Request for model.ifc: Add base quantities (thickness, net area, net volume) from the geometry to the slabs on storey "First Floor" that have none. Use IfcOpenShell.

First a look at what the model holds.

```python
import ifcopenshell
import ifcopenshell.util.element
import ifcopenshell.util.unit

model = ifcopenshell.open("model.ifc")
print(model.schema)
for unit_type in ("LENGTHUNIT", "AREAUNIT", "VOLUMEUNIT"):
    print(unit_type, ifcopenshell.util.unit.calculate_unit_scale(model, unit_type))
storey = next(s for s in model.by_type("IfcBuildingStorey") if s.Name == "First Floor")
slabs = [e for e in ifcopenshell.util.element.get_decomposition(storey) if e.is_a("IfcSlab")]
for e in sorted(slabs, key=lambda e: e.id()):
    print(e.id(), e.is_a(), e.Name, list(ifcopenshell.util.element.get_psets(e, qtos_only=True)), sep=" | ")
```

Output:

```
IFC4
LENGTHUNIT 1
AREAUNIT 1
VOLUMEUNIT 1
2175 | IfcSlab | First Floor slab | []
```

```python
import ifcopenshell
import ifcopenshell.api.pset
import ifcopenshell.geom
import ifcopenshell.util.element
import ifcopenshell.util.shape
import ifcopenshell.util.unit

model = ifcopenshell.open("model.ifc")
unit_scale = ifcopenshell.util.unit.calculate_unit_scale(model)
area_scale = ifcopenshell.util.unit.calculate_unit_scale(model, "AREAUNIT")
volume_scale = ifcopenshell.util.unit.calculate_unit_scale(model, "VOLUMEUNIT")
settings = ifcopenshell.geom.settings()

storey = next(s for s in model.by_type("IfcBuildingStorey") if s.Name == "First Floor")
slabs = [e for e in ifcopenshell.util.element.get_decomposition(storey) if e.is_a("IfcSlab")]

for e in sorted(slabs, key=lambda e: e.id()):
    if ifcopenshell.util.element.get_psets(e, qtos_only=True, should_inherit=False):
        continue
    # Geometry comes back in metres, in the element's own axes.
    shape = ifcopenshell.geom.create_shape(settings, e)
    values = {
        "Width": ifcopenshell.util.shape.get_z(shape.geometry) / unit_scale,
        "NetArea": ifcopenshell.util.shape.get_footprint_area(shape.geometry) / area_scale,
        "NetVolume": ifcopenshell.util.shape.get_volume(shape.geometry) / volume_scale,
    }
    qto = ifcopenshell.api.pset.add_qto(model, product=e, name="Qto_SlabBaseQuantities")
    ifcopenshell.api.pset.edit_qto(model, qto=qto, properties=values)
    print(e.id(), {k: round(v, 3) for k, v in values.items()})

model.write("model_rev.ifc")
```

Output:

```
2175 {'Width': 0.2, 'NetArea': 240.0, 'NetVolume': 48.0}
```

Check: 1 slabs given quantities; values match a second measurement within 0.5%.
